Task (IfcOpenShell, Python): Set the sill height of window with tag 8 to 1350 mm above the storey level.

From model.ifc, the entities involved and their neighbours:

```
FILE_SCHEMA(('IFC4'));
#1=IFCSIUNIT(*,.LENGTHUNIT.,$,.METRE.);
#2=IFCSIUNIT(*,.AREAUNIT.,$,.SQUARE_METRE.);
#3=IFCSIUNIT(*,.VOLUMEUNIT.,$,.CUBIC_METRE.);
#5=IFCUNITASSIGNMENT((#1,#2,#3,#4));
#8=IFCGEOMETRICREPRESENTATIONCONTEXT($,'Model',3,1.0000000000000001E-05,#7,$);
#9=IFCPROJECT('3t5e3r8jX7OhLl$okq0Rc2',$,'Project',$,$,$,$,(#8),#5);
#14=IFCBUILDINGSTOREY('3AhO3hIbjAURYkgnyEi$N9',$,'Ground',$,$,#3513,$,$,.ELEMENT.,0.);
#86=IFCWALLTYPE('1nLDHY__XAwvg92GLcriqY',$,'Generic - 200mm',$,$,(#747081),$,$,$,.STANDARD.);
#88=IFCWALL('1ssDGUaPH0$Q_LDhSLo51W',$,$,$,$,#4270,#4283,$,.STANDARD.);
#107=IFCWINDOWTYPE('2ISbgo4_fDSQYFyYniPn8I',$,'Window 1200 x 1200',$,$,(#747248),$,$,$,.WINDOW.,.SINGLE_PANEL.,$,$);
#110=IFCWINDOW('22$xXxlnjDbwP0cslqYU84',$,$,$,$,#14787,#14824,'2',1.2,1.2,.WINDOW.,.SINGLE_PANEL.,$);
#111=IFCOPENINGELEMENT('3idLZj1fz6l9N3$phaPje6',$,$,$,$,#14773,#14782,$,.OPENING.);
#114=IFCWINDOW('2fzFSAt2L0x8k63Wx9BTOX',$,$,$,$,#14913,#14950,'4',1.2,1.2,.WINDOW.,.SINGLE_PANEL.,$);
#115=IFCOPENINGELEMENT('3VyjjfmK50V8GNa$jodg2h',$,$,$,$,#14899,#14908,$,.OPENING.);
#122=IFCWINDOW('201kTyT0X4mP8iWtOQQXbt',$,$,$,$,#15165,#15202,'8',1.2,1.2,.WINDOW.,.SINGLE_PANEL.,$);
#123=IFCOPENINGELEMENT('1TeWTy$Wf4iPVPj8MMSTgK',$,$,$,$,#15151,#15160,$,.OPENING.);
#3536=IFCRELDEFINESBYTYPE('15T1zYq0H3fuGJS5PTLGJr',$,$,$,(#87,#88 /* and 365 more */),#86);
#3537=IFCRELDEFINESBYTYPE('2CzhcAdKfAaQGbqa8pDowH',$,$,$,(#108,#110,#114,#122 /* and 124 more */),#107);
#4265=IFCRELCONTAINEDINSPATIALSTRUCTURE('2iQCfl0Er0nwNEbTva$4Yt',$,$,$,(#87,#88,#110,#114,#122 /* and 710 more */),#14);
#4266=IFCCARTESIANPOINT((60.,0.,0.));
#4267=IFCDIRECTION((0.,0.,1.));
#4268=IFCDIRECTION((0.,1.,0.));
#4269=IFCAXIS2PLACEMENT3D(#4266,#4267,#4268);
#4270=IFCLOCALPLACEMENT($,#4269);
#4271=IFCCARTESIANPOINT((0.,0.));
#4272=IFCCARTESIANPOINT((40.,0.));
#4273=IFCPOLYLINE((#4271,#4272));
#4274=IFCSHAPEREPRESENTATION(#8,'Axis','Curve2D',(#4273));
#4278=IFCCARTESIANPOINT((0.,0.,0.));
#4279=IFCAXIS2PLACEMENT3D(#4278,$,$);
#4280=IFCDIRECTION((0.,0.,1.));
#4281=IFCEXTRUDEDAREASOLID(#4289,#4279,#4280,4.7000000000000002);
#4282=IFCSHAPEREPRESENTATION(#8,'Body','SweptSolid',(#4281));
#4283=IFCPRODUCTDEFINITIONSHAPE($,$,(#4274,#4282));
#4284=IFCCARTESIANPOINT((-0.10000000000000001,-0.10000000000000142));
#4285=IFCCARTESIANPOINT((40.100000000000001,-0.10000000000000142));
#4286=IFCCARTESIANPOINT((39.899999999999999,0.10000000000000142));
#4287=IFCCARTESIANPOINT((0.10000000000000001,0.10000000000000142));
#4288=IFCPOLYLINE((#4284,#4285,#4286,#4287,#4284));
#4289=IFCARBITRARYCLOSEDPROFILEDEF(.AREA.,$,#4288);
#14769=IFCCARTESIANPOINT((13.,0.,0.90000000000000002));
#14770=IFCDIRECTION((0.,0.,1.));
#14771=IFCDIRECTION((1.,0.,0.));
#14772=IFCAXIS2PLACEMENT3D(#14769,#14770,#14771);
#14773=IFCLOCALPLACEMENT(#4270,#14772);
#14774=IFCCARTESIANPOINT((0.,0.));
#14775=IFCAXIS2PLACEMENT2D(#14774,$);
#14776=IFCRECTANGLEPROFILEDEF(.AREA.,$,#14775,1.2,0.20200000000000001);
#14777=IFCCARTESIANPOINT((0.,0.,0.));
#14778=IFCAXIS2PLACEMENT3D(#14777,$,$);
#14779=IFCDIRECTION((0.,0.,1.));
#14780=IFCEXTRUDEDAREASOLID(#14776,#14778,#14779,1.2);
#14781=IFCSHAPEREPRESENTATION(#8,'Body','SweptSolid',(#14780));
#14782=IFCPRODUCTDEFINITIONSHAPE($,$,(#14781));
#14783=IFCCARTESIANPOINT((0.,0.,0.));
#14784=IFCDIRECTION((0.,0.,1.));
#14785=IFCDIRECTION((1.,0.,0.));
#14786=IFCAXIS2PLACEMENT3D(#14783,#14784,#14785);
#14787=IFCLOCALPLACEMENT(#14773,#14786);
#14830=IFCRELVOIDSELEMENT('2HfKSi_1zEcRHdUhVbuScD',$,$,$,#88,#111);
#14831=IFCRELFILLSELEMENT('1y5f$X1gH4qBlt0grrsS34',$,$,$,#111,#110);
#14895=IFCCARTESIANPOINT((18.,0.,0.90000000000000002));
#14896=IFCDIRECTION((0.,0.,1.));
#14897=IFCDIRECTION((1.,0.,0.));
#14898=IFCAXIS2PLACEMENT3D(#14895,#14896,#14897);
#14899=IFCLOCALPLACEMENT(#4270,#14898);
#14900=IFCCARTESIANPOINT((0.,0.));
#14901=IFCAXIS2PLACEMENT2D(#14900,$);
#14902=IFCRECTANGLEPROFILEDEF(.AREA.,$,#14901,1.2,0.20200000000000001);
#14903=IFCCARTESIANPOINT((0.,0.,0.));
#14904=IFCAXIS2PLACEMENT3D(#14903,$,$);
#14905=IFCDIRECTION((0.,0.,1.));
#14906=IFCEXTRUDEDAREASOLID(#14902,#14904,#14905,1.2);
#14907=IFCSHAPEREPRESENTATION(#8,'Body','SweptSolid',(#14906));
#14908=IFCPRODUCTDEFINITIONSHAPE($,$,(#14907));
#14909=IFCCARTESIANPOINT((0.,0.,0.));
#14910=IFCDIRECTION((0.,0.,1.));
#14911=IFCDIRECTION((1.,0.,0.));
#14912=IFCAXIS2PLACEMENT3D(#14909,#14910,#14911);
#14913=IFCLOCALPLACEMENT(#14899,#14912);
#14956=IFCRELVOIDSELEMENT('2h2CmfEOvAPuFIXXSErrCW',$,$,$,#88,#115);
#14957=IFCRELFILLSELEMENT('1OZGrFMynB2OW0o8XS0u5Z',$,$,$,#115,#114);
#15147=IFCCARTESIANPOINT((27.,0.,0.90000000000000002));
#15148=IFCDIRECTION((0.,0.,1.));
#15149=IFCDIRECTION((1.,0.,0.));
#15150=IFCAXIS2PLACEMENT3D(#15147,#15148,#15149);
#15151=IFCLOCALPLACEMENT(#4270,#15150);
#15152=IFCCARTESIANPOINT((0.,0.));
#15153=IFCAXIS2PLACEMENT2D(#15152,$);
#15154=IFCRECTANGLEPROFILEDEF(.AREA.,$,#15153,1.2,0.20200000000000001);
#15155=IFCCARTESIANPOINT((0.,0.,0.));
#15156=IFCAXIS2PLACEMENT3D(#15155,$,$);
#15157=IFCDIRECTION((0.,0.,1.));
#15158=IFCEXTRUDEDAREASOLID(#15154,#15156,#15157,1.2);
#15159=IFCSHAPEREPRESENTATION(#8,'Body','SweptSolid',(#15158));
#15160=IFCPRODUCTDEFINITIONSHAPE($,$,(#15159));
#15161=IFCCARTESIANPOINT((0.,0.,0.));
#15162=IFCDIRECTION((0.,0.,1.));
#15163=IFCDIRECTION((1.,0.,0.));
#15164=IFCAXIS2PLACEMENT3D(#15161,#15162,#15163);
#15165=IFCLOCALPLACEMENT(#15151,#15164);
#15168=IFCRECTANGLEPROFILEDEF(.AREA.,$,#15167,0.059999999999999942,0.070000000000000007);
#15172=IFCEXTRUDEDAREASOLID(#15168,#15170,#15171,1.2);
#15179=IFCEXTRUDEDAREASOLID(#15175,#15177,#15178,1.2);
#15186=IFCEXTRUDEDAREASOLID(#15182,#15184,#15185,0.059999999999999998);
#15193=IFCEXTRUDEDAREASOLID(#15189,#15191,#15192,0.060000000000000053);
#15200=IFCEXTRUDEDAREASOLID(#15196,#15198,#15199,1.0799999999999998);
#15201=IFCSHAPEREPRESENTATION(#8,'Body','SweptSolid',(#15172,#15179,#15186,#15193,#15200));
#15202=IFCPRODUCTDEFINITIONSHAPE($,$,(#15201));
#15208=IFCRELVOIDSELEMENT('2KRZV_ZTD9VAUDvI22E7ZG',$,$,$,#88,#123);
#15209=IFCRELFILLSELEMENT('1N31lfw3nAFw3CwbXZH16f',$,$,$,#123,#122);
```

```python
import numpy as np
import ifcopenshell
import ifcopenshell.api.geometry
import ifcopenshell.geom
import ifcopenshell.util.element
import ifcopenshell.util.placement
import ifcopenshell.util.shape
import ifcopenshell.util.unit

model = ifcopenshell.open("model.ifc")
unit_scale = ifcopenshell.util.unit.calculate_unit_scale(model)

window = model.by_guid("201kTyT0X4mP8iWtOQQXbt")
opening = window.FillsVoids[0].RelatingOpeningElement
storey = ifcopenshell.util.element.get_container(window, ifc_class="IfcBuildingStorey")
level = ifcopenshell.util.placement.get_local_placement(storey.ObjectPlacement)[2, 3]

# The opening's origin need not be at the sill, so measure its lowest point.
shape = ifcopenshell.geom.create_shape(ifcopenshell.geom.settings(), opening)
bottom = ifcopenshell.util.shape.get_shape_bottom_elevation(shape, shape.geometry) / unit_scale
dz = level + 1.35 - bottom

shift = np.array([0.0, 0.0, dz])
# The window is placed relative to its opening, so it follows when the opening moves.
matrix = ifcopenshell.util.placement.get_local_placement(opening.ObjectPlacement)
matrix[:3, 3] += shift
ifcopenshell.api.geometry.edit_object_placement(
    model, product=opening, matrix=matrix, is_si=False, should_transform_children=True
)

print(f"moved by {dz * unit_scale:+.3f} m")

model.write("model_edited.ifc")
```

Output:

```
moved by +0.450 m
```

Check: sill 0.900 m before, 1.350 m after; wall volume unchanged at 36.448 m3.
